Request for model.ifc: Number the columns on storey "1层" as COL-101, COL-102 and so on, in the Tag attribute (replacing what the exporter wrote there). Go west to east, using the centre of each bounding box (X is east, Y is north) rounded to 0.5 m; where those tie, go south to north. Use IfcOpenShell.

First a look at what the model holds.

```python
import ifcopenshell
import ifcopenshell.util.element
import ifcopenshell.util.placement

model = ifcopenshell.open("model.ifc")
print(model.schema)
storey = next(s for s in model.by_type("IfcBuildingStorey") if s.Name == "1层")
columns = [e for e in ifcopenshell.util.element.get_decomposition(storey) if e.is_a("IfcColumn")]
for e in sorted(columns, key=lambda e: e.id()):
    origin = ifcopenshell.util.placement.get_local_placement(e.ObjectPlacement)[:3, 3]
    print(e.id(), e.Tag, e.Name, origin.round(2) + 0.0, sep=" | ")
```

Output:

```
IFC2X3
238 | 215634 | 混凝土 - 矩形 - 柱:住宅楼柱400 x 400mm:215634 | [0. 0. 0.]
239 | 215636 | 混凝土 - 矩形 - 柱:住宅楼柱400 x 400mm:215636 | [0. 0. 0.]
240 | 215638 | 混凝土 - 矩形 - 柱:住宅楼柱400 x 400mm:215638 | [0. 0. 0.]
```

```python
import ifcopenshell
import ifcopenshell.geom
import ifcopenshell.util.element
import ifcopenshell.util.shape

model = ifcopenshell.open("model.ifc")
settings = ifcopenshell.geom.settings()
settings.set("use-world-coords", True)


def centre(element):
    shape = ifcopenshell.geom.create_shape(settings, element)
    return ifcopenshell.util.shape.get_bbox_centroid(shape.geometry)


storey = next(s for s in model.by_type("IfcBuildingStorey") if s.Name == "1层")
columns = [e for e in ifcopenshell.util.element.get_decomposition(storey) if e.is_a("IfcColumn")]

# Insertion points can sit at a corner or the storey origin, so sort by the geometry (in metres).
centres = {e: centre(e) for e in columns}
columns.sort(key=lambda e: (round(centres[e][0] / 0.5), centres[e][1]))

for i, e in enumerate(columns, start=1):
    number = f"COL-1{i:02d}"
    e.Tag = number
    print(e.id(), number)

model.write("model_updated.ifc")
```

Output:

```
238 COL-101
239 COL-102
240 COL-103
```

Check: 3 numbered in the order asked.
